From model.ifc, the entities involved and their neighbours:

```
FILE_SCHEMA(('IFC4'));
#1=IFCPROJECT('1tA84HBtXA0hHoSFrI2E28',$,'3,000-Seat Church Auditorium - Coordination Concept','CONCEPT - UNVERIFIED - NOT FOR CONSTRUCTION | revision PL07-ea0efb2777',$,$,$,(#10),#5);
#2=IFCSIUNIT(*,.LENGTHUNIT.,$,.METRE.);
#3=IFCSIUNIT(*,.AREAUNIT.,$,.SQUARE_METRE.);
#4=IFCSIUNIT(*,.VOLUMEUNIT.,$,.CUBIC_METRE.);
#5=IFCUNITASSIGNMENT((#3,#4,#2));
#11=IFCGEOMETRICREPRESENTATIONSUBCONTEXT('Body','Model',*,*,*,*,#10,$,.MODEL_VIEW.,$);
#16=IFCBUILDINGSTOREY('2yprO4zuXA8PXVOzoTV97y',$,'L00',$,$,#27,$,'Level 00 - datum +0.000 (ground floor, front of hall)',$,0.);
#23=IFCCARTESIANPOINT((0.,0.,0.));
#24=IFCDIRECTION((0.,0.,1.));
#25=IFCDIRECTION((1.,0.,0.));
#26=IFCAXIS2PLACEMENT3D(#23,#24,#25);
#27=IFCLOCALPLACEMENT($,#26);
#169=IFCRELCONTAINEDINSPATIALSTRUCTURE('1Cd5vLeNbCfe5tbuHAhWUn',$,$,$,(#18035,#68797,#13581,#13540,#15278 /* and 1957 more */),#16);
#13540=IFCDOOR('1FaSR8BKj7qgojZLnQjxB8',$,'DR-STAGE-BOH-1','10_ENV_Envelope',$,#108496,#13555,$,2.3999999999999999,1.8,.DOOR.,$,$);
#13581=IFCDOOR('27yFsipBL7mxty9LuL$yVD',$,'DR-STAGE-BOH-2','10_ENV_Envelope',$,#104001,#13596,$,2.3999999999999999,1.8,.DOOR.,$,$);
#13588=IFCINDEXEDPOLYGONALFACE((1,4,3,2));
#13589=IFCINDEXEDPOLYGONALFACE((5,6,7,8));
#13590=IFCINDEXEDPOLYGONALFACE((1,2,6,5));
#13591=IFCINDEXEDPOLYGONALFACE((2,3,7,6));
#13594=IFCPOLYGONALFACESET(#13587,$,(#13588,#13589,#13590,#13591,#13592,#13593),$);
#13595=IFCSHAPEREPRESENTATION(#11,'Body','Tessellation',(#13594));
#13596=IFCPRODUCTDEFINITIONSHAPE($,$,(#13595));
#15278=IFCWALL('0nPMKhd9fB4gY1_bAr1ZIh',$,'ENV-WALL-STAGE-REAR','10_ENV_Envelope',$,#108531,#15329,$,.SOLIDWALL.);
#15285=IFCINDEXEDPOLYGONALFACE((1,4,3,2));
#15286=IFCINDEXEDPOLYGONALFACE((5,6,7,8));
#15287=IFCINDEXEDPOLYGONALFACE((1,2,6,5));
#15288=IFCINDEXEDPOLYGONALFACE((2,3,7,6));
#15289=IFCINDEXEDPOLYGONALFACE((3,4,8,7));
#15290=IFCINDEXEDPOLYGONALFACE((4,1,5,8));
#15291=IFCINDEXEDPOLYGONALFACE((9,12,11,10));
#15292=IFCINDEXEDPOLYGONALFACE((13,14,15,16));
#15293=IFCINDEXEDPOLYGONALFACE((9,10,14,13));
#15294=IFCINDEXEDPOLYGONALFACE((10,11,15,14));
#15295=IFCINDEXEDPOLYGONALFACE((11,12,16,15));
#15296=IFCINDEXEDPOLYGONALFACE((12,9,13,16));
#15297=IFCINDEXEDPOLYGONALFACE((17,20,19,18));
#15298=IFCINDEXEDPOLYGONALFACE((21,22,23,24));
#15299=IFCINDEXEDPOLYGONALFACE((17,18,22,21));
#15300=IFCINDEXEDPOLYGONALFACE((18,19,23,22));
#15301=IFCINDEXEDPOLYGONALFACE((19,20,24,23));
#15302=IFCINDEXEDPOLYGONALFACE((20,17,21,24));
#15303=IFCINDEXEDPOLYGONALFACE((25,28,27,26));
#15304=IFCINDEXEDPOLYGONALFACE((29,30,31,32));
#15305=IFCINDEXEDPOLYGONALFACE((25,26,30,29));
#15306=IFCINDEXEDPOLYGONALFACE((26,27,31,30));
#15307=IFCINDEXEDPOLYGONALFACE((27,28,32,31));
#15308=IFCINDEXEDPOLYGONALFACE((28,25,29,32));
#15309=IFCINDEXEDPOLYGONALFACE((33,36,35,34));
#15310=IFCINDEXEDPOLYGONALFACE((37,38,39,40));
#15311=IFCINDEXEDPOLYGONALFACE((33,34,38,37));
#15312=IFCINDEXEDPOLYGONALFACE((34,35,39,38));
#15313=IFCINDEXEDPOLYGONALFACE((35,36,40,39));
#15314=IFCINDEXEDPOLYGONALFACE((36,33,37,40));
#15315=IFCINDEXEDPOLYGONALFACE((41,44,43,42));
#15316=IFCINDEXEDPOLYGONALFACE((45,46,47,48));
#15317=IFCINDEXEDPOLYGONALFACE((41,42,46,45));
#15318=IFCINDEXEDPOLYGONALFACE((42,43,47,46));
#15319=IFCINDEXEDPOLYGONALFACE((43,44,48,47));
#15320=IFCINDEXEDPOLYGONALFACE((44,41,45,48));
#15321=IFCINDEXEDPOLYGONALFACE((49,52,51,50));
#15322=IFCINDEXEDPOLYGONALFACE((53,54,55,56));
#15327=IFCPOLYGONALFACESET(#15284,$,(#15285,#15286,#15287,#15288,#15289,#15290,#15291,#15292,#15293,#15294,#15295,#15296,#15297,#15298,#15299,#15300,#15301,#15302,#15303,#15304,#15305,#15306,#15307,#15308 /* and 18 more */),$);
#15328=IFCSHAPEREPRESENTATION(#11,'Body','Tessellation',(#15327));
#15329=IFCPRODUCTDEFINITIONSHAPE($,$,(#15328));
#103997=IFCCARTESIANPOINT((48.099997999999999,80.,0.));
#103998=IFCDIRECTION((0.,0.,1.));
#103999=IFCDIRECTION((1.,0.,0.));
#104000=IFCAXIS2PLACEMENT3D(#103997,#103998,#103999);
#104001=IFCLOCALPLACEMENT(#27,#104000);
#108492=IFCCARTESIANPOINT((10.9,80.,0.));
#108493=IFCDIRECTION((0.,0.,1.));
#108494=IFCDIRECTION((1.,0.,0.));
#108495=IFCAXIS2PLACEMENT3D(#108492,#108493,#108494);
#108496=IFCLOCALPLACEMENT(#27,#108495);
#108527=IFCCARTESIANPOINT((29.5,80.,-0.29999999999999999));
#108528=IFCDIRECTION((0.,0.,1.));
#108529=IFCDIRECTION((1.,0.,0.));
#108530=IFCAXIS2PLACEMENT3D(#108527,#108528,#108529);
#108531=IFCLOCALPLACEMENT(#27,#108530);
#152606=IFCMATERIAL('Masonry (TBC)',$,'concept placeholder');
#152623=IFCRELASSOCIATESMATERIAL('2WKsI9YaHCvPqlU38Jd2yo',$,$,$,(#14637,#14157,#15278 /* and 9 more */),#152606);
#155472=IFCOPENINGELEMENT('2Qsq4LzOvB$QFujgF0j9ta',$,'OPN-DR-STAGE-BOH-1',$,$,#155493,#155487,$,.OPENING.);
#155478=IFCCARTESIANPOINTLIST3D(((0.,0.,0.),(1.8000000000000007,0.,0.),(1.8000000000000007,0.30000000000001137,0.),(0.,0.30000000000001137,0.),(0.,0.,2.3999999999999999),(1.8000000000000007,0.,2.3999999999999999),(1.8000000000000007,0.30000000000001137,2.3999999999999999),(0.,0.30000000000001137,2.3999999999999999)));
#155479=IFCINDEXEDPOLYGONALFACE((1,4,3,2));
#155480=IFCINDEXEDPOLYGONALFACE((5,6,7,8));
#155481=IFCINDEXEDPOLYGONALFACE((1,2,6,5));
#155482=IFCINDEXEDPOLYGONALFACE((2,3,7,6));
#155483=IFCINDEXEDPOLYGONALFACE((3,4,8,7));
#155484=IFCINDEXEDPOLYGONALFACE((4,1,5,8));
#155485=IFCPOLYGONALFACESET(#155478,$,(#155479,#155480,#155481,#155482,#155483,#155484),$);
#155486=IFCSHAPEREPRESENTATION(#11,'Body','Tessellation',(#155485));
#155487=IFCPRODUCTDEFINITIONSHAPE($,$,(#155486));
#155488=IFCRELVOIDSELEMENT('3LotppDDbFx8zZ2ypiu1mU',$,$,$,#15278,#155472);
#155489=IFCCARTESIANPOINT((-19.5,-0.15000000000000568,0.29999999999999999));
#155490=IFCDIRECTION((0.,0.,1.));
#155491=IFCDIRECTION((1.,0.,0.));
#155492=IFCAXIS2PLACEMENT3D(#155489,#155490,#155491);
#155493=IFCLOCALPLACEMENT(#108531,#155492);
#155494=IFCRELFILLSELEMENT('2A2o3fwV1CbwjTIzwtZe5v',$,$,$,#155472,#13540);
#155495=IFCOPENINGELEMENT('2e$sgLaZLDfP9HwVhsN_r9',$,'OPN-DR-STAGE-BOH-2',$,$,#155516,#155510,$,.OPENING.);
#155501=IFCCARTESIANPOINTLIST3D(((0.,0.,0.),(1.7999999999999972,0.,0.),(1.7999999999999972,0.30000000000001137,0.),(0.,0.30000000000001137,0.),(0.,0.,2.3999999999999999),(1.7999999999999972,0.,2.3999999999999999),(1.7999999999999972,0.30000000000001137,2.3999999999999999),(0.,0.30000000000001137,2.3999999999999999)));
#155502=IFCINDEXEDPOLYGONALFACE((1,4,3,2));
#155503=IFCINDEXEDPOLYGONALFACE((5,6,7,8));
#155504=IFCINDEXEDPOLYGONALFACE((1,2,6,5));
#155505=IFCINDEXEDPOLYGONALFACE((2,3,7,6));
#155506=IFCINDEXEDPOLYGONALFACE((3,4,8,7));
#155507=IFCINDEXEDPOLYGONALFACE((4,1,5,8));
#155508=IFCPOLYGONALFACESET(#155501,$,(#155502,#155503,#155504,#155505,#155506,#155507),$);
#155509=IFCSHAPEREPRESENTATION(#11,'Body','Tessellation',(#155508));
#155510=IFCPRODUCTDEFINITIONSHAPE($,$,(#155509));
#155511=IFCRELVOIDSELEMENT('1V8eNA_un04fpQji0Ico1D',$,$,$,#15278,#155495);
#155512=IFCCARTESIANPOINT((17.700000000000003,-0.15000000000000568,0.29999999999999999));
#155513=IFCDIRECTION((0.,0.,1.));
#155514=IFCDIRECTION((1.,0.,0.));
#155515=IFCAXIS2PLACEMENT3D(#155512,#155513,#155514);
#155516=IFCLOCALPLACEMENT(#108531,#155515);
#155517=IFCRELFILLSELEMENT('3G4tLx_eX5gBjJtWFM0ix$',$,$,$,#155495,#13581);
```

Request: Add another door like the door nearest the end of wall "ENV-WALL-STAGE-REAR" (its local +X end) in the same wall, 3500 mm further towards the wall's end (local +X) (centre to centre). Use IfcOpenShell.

```python
import ifcopenshell
import ifcopenshell.api.feature
import ifcopenshell.api.geometry
import ifcopenshell.api.root
import ifcopenshell.geom
import ifcopenshell.util.element
import ifcopenshell.util.placement
import ifcopenshell.util.shape

model = ifcopenshell.open("model.ifc")
settings = ifcopenshell.geom.settings()


def volume(element):
    """Net volume in cubic metres, openings subtracted."""
    shape = ifcopenshell.geom.create_shape(settings, element)
    return ifcopenshell.util.shape.get_volume(shape.geometry)


door = model.by_guid("27yFsipBL7mxty9LuL$yVD")
opening = door.FillsVoids[0].RelatingOpeningElement
wall = opening.VoidsElements[0].RelatingBuildingElement
before = volume(wall)
shift = ifcopenshell.util.placement.get_local_placement(wall.ObjectPlacement)[:3, 0] * 3.5

# copy_class copies the void relationship, type, container and properties, but no geometry.
new_opening = ifcopenshell.api.root.copy_class(model, product=opening)
new_opening.Representation = ifcopenshell.util.element.copy_deep(
    model, opening.Representation, exclude=["IfcGeometricRepresentationContext", "IfcRepresentationMap"]
)
new_door = ifcopenshell.api.root.copy_class(model, product=door)
new_door.Representation = ifcopenshell.util.element.copy_deep(
    model, door.Representation, exclude=["IfcGeometricRepresentationContext", "IfcRepresentationMap"]
)
ifcopenshell.api.feature.add_filling(model, opening=new_opening, element=new_door)

for old, new in ((opening, new_opening), (door, new_door)):
    matrix = ifcopenshell.util.placement.get_local_placement(old.ObjectPlacement)
    matrix[:3, 3] += shift
    ifcopenshell.api.geometry.edit_object_placement(model, product=new, matrix=matrix, is_si=False)

after = volume(wall)

print(f"wall volume {before:.3f} -> {after:.3f} m3")

model.write("model_rev.ifc")
```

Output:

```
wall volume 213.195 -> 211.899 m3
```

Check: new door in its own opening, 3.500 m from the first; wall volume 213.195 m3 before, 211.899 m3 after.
